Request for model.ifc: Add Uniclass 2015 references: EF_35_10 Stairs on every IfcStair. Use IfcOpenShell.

First a look at what the model holds.

```python
import ifcopenshell

model = ifcopenshell.open("model.ifc")
print(model.schema)
print("classifications:", [c.Name for c in model.by_type("IfcClassification")])
for ifc_class in ("IfcDoor", "IfcRoof", "IfcStair", "IfcWall", "IfcWindow"):
    print(ifc_class, len(model.by_type(ifc_class)))
```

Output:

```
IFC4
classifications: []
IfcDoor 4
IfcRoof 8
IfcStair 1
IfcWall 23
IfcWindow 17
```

```python
import ifcopenshell
import ifcopenshell.api.classification

model = ifcopenshell.open("model.ifc")

system = ifcopenshell.api.classification.add_classification(model, classification="Uniclass 2015")

codes = {
    "IfcStair": ("EF_35_10", "Stairs"),
}
for ifc_class, (code, name) in codes.items():
    products = model.by_type(ifc_class)
    ifcopenshell.api.classification.add_reference(
        model, products=products, classification=system, identification=code, name=name
    )
    print(code, len(products))

model.write("model_edited.ifc")
```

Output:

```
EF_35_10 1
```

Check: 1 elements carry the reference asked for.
